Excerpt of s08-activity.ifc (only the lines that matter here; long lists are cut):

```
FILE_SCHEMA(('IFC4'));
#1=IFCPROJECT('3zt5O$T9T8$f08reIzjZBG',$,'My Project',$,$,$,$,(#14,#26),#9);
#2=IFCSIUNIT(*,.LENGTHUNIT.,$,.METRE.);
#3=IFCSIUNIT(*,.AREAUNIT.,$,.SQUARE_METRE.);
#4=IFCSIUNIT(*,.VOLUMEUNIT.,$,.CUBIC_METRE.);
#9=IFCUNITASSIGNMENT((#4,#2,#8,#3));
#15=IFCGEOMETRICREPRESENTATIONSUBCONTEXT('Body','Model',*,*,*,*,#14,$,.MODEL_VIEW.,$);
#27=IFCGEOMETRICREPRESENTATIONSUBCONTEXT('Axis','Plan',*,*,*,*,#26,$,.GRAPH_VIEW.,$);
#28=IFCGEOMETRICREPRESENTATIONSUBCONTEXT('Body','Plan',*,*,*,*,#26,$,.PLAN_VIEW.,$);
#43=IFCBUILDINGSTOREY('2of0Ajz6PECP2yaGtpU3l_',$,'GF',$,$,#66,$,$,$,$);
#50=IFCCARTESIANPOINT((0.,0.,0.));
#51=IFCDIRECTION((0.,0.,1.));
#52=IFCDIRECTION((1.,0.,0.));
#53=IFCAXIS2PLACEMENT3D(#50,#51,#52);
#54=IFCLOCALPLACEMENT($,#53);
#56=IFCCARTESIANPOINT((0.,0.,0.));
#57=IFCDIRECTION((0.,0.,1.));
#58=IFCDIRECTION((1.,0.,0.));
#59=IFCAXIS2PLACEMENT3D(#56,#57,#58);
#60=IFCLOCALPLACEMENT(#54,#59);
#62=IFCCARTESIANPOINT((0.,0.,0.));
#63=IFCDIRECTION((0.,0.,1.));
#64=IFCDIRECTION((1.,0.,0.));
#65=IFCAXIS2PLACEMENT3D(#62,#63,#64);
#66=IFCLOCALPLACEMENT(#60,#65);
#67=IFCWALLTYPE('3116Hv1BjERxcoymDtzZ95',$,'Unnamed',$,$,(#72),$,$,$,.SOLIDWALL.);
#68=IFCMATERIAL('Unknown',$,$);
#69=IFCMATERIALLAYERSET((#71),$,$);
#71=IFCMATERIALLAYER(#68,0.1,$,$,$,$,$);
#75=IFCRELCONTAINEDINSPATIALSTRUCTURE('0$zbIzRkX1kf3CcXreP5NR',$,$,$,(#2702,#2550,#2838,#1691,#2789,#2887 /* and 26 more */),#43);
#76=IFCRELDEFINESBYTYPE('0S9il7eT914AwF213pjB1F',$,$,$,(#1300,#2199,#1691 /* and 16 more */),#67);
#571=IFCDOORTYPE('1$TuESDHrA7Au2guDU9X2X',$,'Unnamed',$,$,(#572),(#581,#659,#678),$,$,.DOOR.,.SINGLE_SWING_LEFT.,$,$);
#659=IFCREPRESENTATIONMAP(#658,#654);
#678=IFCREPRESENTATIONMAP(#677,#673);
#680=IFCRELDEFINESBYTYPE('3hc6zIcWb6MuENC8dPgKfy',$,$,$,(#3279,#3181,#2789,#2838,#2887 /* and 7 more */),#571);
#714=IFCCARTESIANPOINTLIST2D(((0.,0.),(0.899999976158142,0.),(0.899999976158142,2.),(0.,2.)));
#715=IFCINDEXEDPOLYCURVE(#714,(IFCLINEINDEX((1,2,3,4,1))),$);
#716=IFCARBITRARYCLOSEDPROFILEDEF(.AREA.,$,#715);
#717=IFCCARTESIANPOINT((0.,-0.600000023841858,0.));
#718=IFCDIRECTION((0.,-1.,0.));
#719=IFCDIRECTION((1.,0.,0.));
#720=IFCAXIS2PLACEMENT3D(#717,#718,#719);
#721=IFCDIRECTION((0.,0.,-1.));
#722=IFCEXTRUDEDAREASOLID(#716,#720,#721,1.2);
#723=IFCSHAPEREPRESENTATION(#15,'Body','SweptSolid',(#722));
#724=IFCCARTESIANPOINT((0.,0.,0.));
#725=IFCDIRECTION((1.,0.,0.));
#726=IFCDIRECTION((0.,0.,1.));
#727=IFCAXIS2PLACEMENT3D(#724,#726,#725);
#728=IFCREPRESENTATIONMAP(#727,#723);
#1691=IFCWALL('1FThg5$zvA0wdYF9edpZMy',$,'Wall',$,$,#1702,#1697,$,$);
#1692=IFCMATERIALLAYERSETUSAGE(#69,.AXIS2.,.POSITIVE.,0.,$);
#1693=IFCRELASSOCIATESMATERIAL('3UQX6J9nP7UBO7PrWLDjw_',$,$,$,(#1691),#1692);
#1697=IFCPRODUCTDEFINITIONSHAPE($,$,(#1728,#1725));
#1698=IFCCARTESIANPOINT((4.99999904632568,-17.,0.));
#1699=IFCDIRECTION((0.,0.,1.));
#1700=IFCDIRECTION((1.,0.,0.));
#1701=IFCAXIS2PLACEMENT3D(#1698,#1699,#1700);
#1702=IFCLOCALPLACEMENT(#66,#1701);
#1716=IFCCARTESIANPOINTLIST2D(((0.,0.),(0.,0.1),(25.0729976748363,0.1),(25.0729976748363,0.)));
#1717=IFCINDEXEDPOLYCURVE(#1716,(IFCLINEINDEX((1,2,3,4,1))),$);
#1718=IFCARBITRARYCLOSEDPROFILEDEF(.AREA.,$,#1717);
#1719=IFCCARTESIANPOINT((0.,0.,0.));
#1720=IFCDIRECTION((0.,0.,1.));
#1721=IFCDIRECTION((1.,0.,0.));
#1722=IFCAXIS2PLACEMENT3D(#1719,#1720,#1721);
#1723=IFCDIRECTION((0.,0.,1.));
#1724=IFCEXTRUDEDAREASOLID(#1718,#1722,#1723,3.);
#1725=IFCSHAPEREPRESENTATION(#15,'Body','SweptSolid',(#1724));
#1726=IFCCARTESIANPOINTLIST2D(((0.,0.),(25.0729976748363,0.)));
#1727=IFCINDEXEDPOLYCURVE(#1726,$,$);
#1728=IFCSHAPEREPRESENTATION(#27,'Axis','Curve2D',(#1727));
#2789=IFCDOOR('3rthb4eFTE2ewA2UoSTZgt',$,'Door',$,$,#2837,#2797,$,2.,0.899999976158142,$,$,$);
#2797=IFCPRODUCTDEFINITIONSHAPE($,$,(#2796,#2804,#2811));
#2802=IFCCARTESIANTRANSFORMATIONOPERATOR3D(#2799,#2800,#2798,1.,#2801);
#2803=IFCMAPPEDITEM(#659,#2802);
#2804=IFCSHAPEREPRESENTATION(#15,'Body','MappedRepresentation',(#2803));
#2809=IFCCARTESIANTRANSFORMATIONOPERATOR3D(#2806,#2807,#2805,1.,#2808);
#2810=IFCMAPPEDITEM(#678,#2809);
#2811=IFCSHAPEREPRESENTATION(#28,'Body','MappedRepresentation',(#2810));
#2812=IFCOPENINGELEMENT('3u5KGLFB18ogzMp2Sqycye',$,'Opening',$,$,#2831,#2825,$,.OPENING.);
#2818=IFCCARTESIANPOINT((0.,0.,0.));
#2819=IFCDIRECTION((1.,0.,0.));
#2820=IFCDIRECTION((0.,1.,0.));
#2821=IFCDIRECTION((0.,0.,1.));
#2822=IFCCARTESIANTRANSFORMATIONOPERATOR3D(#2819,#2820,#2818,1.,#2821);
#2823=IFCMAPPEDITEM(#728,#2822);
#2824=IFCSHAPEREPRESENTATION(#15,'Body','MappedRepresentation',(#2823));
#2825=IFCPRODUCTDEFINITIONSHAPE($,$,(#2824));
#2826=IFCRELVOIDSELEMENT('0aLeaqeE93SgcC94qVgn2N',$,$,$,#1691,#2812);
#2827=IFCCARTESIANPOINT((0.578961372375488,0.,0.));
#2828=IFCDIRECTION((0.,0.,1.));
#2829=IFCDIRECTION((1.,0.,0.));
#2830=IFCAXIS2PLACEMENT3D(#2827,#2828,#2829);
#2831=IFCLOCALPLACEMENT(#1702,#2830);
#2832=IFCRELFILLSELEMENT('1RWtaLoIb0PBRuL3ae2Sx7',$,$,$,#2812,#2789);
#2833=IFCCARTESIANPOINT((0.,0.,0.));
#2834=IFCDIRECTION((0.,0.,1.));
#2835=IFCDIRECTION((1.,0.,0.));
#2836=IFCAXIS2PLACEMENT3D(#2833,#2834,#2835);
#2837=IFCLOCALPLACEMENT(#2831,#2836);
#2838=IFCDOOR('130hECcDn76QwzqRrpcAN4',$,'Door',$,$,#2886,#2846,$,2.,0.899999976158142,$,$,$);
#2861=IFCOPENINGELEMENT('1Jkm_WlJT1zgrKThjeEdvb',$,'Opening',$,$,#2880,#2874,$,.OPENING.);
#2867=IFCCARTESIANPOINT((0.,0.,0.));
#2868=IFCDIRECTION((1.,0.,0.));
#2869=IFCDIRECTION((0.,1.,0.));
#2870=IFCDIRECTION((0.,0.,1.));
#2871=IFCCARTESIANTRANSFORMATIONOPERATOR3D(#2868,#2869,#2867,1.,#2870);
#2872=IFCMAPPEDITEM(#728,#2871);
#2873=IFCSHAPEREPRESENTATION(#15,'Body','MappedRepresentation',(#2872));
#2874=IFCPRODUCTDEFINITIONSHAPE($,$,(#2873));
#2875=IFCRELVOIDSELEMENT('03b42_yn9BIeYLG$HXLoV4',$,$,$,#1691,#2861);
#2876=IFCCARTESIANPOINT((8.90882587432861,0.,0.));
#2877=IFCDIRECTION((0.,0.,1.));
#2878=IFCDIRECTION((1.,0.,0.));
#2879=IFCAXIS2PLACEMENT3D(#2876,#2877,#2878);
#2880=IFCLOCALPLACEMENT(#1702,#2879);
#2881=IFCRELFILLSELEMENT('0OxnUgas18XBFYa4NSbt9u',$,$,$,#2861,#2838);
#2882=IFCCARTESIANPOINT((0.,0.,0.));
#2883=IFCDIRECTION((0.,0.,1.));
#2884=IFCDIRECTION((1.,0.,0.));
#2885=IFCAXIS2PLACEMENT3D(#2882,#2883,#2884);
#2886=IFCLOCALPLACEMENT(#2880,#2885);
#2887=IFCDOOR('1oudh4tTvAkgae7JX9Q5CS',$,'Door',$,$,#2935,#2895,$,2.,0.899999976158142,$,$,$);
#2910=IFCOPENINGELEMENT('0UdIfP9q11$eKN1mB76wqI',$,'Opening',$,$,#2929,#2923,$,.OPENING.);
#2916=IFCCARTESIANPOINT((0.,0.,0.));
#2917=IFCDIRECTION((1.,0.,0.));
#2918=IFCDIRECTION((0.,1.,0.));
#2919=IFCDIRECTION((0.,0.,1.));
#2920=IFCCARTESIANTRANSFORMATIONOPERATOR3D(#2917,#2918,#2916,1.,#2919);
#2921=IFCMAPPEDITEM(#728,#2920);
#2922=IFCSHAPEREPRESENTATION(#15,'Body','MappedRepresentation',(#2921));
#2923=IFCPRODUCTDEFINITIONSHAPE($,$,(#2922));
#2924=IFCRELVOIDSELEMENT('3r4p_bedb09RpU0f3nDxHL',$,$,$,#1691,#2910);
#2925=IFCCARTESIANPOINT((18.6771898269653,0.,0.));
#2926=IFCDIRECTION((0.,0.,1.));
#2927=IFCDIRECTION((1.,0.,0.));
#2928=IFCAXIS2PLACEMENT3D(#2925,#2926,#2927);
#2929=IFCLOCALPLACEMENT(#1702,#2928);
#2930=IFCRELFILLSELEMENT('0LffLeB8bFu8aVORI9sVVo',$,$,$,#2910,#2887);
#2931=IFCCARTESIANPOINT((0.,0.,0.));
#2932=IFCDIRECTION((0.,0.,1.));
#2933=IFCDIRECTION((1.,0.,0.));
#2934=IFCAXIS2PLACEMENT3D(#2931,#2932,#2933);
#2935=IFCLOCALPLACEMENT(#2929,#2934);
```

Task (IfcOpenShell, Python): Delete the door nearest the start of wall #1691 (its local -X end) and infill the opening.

```python
import ifcopenshell
import ifcopenshell.api.feature
import ifcopenshell.api.root
import ifcopenshell.geom
import ifcopenshell.util.shape

model = ifcopenshell.open("s08-activity.ifc")
settings = ifcopenshell.geom.settings()


def volume(element):
    """Net volume in cubic metres, openings subtracted."""
    shape = ifcopenshell.geom.create_shape(settings, element)
    return ifcopenshell.util.shape.get_volume(shape.geometry)


door = model.by_guid("3rthb4eFTE2ewA2UoSTZgt")
opening = door.FillsVoids[0].RelatingOpeningElement
wall = opening.VoidsElements[0].RelatingBuildingElement
before = volume(wall)

ifcopenshell.api.root.remove_product(model, product=door)
ifcopenshell.api.feature.remove_feature(model, feature=opening)

after = volume(wall)

print(f"wall volume {before:.3f} -> {after:.3f} m3")

model.write("s08-activity_v2.ifc")
```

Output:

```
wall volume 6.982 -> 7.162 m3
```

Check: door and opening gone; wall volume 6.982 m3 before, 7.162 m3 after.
